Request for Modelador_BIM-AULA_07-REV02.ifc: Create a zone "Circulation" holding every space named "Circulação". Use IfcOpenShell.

First a look at what the model holds.

```python
import ifcopenshell

model = ifcopenshell.open("Modelador_BIM-AULA_07-REV02.ifc")
print(model.schema)
seen = {}
for space in model.by_type("IfcSpace"):
    seen[space.LongName] = seen.get(space.LongName, 0) + 1
for name, count in sorted(seen.items(), key=str):
    print(count, "x", name)
print("zones:", [z.Name for z in model.by_type("IfcZone")][:20])
```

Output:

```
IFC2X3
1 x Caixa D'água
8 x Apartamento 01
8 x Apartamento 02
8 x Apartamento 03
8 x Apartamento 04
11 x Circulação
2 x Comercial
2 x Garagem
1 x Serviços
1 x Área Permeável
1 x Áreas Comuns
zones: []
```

```python
import ifcopenshell
import ifcopenshell.api.group
import ifcopenshell.api.root

model = ifcopenshell.open("Modelador_BIM-AULA_07-REV02.ifc")

names = {"Circulação"}
spaces = [s for s in model.by_type("IfcSpace") if s.LongName in names]

zone = ifcopenshell.api.root.create_entity(model, ifc_class="IfcZone", name="Circulation")
ifcopenshell.api.group.assign_group(model, products=spaces, group=zone)
print(len(spaces), "spaces in", zone.Name)

model.write("Modelador_BIM-AULA_07-REV02_edited.ifc")
```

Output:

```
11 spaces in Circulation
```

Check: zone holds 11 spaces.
